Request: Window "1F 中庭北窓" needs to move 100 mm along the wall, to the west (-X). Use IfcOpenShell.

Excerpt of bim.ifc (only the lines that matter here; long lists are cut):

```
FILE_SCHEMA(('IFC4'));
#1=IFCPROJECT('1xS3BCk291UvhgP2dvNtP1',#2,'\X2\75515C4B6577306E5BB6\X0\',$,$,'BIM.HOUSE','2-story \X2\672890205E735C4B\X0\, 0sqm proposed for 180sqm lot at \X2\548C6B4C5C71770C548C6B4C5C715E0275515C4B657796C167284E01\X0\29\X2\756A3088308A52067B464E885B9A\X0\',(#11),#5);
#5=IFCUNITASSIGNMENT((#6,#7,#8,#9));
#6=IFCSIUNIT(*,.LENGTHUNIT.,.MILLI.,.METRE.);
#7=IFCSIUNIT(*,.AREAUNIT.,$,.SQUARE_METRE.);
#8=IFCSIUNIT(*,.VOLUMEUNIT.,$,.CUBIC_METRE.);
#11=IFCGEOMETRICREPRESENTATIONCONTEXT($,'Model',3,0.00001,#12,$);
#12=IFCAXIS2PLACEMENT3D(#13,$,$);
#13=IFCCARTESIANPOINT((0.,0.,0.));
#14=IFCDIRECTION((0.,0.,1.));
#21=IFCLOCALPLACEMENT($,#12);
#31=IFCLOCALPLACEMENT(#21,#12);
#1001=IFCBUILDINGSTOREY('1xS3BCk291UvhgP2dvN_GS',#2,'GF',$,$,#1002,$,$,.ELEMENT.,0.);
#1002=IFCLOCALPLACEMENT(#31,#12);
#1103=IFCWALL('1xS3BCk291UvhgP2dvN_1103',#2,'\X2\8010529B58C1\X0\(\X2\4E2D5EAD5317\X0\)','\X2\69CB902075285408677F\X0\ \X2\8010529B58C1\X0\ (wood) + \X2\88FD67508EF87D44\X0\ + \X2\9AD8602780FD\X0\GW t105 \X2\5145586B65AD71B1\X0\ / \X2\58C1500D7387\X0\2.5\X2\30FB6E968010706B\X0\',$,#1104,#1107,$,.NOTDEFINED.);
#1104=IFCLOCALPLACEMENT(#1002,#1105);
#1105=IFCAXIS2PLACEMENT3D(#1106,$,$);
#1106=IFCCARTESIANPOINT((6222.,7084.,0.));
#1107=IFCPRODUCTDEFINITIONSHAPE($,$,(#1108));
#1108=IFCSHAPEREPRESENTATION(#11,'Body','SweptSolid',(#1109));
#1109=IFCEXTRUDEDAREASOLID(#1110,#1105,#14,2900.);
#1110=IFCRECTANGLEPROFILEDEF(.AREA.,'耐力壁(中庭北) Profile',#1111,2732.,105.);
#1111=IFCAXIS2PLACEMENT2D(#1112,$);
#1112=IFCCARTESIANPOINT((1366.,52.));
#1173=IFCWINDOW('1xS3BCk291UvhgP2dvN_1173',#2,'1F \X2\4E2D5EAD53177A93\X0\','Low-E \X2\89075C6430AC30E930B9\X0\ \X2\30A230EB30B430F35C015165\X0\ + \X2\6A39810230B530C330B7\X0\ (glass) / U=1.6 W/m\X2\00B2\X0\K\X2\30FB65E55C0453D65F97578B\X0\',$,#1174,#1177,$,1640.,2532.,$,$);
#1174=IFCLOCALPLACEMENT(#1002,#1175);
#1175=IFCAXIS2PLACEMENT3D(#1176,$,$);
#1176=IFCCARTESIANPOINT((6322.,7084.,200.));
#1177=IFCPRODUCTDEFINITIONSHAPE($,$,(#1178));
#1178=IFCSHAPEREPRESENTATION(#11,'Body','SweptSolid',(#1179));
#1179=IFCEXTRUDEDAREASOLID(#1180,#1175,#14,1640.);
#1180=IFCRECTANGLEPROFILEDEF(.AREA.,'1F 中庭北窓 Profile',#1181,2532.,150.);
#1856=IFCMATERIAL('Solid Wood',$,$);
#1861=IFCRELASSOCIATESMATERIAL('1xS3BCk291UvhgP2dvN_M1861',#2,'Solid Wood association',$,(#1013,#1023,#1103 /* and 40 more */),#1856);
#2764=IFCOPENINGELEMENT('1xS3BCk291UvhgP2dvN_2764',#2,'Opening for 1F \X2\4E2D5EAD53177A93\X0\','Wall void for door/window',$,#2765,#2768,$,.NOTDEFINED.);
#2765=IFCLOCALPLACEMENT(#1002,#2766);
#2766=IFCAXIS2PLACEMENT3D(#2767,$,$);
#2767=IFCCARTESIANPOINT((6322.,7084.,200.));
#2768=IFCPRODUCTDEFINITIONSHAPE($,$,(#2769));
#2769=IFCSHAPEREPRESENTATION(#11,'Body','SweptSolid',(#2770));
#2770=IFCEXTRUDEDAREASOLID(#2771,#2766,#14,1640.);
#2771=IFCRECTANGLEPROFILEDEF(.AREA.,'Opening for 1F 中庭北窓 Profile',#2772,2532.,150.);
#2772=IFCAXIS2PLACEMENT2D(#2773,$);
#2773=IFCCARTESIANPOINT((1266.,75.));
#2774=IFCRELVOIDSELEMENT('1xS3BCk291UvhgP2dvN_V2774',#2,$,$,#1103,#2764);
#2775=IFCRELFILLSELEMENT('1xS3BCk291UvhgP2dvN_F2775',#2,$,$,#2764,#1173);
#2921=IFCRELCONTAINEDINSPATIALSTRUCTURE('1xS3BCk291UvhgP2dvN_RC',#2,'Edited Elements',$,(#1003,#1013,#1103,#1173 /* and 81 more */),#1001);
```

```python
import ifcopenshell
import ifcopenshell.api.geometry
import ifcopenshell.util.placement
import ifcopenshell.util.unit

model = ifcopenshell.open("bim.ifc")
unit_scale = ifcopenshell.util.unit.calculate_unit_scale(model)

window = model.by_guid("1xS3BCk291UvhgP2dvN_1173")
opening = window.FillsVoids[0].RelatingOpeningElement
wall = opening.VoidsElements[0].RelatingBuildingElement

wall_matrix = ifcopenshell.util.placement.get_local_placement(wall.ObjectPlacement)
shift = wall_matrix[:3, 0] * -0.1 / unit_scale
before = ifcopenshell.util.placement.get_local_placement(window.ObjectPlacement)[:3, 3].copy()

# The window is not placed relative to its opening, so move both.
for product in (opening, window):
    matrix = ifcopenshell.util.placement.get_local_placement(product.ObjectPlacement)
    matrix[:3, 3] += shift
    ifcopenshell.api.geometry.edit_object_placement(model, product=product, matrix=matrix, is_si=False)

after = ifcopenshell.util.placement.get_local_placement(window.ObjectPlacement)[:3, 3]
print("window moved by", (after - before).round(3) + 0.0)

model.write("bim_rev.ifc")
```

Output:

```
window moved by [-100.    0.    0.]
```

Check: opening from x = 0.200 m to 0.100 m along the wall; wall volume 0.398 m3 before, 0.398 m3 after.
